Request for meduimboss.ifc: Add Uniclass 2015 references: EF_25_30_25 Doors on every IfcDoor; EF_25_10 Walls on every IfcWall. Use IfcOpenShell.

First a look at what the model holds.

```python
import ifcopenshell

model = ifcopenshell.open("meduimboss.ifc")
print(model.schema)
print("classifications:", [c.Name for c in model.by_type("IfcClassification")])
for ifc_class in ("IfcDoor", "IfcRoof", "IfcStair", "IfcWall", "IfcWindow"):
    print(ifc_class, len(model.by_type(ifc_class)))
```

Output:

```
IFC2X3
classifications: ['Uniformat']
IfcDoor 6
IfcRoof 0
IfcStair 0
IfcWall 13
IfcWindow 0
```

```python
import ifcopenshell
import ifcopenshell.api.classification

model = ifcopenshell.open("meduimboss.ifc")

# IFC2X3 requires Source and Edition and has no link from the project to the system.
system = model.create_entity("IfcClassification", Source="NBS", Edition="2015", Name="Uniclass 2015")

codes = {
    "IfcDoor": ("EF_25_30_25", "Doors"),
    "IfcWall": ("EF_25_10", "Walls"),
}
for ifc_class, (code, name) in codes.items():
    products = model.by_type(ifc_class)
    ifcopenshell.api.classification.add_reference(
        model, products=products, classification=system, identification=code, name=name
    )
    print(code, len(products))

model.write("meduimboss_v2.ifc")
```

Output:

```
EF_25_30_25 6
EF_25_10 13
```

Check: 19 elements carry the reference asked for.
